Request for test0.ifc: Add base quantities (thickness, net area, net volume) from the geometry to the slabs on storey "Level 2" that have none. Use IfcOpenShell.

First a look at what the model holds.

```python
import ifcopenshell
import ifcopenshell.util.element
import ifcopenshell.util.unit

model = ifcopenshell.open("test0.ifc")
print(model.schema)
for unit_type in ("LENGTHUNIT", "AREAUNIT", "VOLUMEUNIT"):
    print(unit_type, ifcopenshell.util.unit.calculate_unit_scale(model, unit_type))
storey = next(s for s in model.by_type("IfcBuildingStorey") if s.Name == "Level 2")
slabs = [e for e in ifcopenshell.util.element.get_decomposition(storey) if e.is_a("IfcSlab")]
for e in sorted(slabs, key=lambda e: e.id()):
    print(e.id(), e.is_a(), e.Name, list(ifcopenshell.util.element.get_psets(e, qtos_only=True)), sep=" | ")
```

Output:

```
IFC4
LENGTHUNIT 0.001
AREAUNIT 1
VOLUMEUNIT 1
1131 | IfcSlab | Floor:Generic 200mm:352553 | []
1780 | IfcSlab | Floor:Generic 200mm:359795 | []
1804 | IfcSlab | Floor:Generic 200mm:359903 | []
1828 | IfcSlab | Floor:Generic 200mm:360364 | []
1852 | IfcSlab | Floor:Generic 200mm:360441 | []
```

```python
import ifcopenshell
import ifcopenshell.api.pset
import ifcopenshell.geom
import ifcopenshell.util.element
import ifcopenshell.util.shape
import ifcopenshell.util.unit

model = ifcopenshell.open("test0.ifc")
unit_scale = ifcopenshell.util.unit.calculate_unit_scale(model)
area_scale = ifcopenshell.util.unit.calculate_unit_scale(model, "AREAUNIT")
volume_scale = ifcopenshell.util.unit.calculate_unit_scale(model, "VOLUMEUNIT")
settings = ifcopenshell.geom.settings()

storey = next(s for s in model.by_type("IfcBuildingStorey") if s.Name == "Level 2")
slabs = [e for e in ifcopenshell.util.element.get_decomposition(storey) if e.is_a("IfcSlab")]

for e in sorted(slabs, key=lambda e: e.id()):
    if ifcopenshell.util.element.get_psets(e, qtos_only=True, should_inherit=False):
        continue
    # Geometry comes back in metres, in the element's own axes.
    shape = ifcopenshell.geom.create_shape(settings, e)
    values = {
        "Width": ifcopenshell.util.shape.get_z(shape.geometry) / unit_scale,
        "NetArea": ifcopenshell.util.shape.get_footprint_area(shape.geometry) / area_scale,
        "NetVolume": ifcopenshell.util.shape.get_volume(shape.geometry) / volume_scale,
    }
    qto = ifcopenshell.api.pset.add_qto(model, product=e, name="Qto_SlabBaseQuantities")
    ifcopenshell.api.pset.edit_qto(model, qto=qto, properties=values)
    print(e.id(), {k: round(v, 3) for k, v in values.items()})

model.write("test0_v2.ifc")
```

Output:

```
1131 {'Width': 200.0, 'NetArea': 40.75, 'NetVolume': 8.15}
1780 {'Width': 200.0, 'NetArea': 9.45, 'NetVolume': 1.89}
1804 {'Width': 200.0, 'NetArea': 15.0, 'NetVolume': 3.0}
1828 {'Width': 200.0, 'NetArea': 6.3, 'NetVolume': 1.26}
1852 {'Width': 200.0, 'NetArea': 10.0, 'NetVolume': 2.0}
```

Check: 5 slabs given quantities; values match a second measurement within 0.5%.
